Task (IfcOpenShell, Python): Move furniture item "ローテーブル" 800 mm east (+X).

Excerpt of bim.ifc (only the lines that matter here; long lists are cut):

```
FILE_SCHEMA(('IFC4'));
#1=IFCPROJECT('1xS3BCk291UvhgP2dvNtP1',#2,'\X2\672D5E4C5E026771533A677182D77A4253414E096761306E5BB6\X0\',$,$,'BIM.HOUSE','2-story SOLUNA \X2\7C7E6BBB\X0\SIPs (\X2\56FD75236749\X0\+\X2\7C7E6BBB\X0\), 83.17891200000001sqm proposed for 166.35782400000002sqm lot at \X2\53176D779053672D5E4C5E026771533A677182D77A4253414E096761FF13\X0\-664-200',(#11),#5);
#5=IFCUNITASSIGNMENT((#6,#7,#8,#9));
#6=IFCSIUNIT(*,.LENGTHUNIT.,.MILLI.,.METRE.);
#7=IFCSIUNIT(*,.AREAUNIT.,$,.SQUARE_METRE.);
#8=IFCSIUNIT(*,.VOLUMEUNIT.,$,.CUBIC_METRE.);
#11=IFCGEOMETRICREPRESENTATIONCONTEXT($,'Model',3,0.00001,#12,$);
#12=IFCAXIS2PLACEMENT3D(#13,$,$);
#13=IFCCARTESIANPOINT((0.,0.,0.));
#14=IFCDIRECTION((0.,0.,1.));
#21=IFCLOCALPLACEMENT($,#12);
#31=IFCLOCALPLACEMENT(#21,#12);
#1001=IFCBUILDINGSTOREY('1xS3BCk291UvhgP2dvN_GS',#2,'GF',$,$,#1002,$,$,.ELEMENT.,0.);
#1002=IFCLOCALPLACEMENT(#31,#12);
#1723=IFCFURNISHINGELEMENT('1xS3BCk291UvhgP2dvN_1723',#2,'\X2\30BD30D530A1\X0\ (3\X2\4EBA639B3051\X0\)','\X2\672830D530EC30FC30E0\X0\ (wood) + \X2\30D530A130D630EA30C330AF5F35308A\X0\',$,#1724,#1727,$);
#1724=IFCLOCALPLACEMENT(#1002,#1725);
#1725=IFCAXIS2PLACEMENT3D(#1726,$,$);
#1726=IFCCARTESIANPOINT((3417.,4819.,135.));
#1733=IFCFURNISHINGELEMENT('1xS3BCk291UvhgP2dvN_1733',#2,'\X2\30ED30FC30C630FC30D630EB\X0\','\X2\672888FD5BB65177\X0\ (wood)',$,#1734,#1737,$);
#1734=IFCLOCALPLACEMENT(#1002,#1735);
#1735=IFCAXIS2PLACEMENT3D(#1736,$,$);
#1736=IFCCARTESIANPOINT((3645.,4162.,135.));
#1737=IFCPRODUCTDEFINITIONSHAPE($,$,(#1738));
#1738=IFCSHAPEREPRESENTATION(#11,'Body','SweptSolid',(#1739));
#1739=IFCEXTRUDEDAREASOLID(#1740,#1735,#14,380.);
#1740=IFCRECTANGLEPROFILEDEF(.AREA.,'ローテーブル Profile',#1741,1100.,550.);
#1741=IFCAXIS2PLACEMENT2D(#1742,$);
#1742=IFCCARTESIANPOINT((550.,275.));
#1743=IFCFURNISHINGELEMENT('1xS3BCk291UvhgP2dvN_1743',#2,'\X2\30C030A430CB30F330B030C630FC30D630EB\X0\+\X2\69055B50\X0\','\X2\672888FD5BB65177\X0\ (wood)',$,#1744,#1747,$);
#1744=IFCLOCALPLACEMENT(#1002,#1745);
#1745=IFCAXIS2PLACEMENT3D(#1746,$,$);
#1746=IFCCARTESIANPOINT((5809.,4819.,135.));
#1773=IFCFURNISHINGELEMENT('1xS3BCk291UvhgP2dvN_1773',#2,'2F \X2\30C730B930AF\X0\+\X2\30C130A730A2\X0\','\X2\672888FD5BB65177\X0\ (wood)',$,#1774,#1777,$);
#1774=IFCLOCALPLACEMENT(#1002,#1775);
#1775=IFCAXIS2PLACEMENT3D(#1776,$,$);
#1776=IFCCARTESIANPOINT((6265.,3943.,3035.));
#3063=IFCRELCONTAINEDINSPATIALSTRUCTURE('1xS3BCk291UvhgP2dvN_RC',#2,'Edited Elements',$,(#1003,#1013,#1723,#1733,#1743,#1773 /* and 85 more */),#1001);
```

```python
import ifcopenshell
import ifcopenshell.api.geometry
import ifcopenshell.util.placement

model = ifcopenshell.open("bim.ifc")

item = model.by_id(1733)
matrix = ifcopenshell.util.placement.get_local_placement(item.ObjectPlacement)
matrix[0, 3] += 800.0
ifcopenshell.api.geometry.edit_object_placement(model, product=item, matrix=matrix, is_si=False)

print(ifcopenshell.util.placement.get_local_placement(item.ObjectPlacement).round(3) + 0.0)

model.write("bim_v2.ifc")
```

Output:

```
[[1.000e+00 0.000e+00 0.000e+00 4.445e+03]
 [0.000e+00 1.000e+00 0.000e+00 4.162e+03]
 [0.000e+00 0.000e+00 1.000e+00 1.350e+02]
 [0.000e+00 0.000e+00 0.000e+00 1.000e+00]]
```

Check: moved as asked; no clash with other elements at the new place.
